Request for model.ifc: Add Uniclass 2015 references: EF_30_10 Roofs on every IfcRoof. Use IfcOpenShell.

First a look at what the model holds.

```python
import ifcopenshell

model = ifcopenshell.open("model.ifc")
print(model.schema)
print("classifications:", [c.Name for c in model.by_type("IfcClassification")])
for ifc_class in ("IfcDoor", "IfcRoof", "IfcStair", "IfcWall", "IfcWindow"):
    print(ifc_class, len(model.by_type(ifc_class)))
```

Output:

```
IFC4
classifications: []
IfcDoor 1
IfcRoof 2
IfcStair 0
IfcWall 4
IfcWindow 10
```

```python
import ifcopenshell
import ifcopenshell.api.classification

model = ifcopenshell.open("model.ifc")

system = ifcopenshell.api.classification.add_classification(model, classification="Uniclass 2015")

codes = {
    "IfcRoof": ("EF_30_10", "Roofs"),
}
for ifc_class, (code, name) in codes.items():
    products = model.by_type(ifc_class)
    ifcopenshell.api.classification.add_reference(
        model, products=products, classification=system, identification=code, name=name
    )
    print(code, len(products))

model.write("model_rev.ifc")
```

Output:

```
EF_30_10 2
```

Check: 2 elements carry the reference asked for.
